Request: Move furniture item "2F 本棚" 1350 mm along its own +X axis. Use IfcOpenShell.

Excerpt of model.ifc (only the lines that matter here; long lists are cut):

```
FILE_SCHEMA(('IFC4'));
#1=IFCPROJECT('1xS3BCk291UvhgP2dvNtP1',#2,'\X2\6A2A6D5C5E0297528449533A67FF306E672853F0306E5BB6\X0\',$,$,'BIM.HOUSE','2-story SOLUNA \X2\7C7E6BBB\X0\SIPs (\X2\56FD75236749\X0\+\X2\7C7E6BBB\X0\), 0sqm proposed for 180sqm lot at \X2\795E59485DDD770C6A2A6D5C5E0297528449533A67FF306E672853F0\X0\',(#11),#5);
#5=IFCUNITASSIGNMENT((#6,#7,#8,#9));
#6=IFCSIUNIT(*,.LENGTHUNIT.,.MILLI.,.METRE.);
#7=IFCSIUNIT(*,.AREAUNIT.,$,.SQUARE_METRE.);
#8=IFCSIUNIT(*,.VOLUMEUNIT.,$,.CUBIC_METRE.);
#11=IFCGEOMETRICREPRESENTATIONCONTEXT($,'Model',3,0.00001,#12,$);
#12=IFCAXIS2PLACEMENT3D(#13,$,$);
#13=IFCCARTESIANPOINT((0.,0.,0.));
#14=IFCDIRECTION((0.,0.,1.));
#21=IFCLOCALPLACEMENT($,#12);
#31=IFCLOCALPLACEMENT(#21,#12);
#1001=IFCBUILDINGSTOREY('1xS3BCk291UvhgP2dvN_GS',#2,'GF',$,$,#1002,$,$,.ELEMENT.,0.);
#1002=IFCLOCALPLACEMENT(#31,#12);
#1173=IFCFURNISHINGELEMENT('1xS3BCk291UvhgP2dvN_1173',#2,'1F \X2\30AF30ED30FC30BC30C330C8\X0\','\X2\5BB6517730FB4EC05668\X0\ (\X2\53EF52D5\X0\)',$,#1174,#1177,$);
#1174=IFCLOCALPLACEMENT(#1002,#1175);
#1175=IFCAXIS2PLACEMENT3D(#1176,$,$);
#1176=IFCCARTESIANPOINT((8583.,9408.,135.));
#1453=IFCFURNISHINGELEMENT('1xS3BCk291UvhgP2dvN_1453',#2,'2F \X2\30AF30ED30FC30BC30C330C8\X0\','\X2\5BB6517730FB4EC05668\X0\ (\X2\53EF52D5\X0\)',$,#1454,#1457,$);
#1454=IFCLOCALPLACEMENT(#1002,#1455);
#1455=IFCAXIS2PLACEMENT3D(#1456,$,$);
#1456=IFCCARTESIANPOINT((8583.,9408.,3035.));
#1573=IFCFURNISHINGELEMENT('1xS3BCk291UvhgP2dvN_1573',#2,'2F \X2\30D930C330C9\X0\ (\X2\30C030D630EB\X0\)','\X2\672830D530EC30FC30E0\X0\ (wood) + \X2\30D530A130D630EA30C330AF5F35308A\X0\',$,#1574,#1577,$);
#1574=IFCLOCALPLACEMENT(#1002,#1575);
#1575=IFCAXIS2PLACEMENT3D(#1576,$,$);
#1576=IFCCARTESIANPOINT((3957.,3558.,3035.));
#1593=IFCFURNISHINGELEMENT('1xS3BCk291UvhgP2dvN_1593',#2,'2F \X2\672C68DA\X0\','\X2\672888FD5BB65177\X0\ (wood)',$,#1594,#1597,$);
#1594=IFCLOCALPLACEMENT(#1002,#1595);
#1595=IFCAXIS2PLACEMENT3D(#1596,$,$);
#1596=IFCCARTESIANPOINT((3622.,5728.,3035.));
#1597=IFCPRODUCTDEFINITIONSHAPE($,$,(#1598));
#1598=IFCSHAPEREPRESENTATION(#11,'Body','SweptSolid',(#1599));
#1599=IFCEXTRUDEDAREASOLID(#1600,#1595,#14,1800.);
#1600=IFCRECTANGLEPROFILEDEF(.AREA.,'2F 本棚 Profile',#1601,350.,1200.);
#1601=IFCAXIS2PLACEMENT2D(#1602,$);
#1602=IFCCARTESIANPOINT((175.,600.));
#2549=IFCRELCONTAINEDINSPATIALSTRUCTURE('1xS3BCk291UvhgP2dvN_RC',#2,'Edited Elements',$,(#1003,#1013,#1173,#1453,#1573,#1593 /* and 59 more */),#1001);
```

```python
import ifcopenshell
import ifcopenshell.api.geometry
import ifcopenshell.util.placement
import ifcopenshell.util.unit

model = ifcopenshell.open("model.ifc")
unit_scale = ifcopenshell.util.unit.calculate_unit_scale(model)

item = model.by_guid("1xS3BCk291UvhgP2dvN_1593")
matrix = ifcopenshell.util.placement.get_local_placement(item.ObjectPlacement)
matrix[:3, 3] += matrix[:3, 0] * 1.35 / unit_scale
ifcopenshell.api.geometry.edit_object_placement(model, product=item, matrix=matrix, is_si=False)

print(ifcopenshell.util.placement.get_local_placement(item.ObjectPlacement).round(3) + 0.0)

model.write("model_v2.ifc")
```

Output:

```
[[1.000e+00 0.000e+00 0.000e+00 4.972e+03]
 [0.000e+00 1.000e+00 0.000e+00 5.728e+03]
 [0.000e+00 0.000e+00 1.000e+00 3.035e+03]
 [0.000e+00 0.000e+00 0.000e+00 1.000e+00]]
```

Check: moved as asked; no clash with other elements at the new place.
